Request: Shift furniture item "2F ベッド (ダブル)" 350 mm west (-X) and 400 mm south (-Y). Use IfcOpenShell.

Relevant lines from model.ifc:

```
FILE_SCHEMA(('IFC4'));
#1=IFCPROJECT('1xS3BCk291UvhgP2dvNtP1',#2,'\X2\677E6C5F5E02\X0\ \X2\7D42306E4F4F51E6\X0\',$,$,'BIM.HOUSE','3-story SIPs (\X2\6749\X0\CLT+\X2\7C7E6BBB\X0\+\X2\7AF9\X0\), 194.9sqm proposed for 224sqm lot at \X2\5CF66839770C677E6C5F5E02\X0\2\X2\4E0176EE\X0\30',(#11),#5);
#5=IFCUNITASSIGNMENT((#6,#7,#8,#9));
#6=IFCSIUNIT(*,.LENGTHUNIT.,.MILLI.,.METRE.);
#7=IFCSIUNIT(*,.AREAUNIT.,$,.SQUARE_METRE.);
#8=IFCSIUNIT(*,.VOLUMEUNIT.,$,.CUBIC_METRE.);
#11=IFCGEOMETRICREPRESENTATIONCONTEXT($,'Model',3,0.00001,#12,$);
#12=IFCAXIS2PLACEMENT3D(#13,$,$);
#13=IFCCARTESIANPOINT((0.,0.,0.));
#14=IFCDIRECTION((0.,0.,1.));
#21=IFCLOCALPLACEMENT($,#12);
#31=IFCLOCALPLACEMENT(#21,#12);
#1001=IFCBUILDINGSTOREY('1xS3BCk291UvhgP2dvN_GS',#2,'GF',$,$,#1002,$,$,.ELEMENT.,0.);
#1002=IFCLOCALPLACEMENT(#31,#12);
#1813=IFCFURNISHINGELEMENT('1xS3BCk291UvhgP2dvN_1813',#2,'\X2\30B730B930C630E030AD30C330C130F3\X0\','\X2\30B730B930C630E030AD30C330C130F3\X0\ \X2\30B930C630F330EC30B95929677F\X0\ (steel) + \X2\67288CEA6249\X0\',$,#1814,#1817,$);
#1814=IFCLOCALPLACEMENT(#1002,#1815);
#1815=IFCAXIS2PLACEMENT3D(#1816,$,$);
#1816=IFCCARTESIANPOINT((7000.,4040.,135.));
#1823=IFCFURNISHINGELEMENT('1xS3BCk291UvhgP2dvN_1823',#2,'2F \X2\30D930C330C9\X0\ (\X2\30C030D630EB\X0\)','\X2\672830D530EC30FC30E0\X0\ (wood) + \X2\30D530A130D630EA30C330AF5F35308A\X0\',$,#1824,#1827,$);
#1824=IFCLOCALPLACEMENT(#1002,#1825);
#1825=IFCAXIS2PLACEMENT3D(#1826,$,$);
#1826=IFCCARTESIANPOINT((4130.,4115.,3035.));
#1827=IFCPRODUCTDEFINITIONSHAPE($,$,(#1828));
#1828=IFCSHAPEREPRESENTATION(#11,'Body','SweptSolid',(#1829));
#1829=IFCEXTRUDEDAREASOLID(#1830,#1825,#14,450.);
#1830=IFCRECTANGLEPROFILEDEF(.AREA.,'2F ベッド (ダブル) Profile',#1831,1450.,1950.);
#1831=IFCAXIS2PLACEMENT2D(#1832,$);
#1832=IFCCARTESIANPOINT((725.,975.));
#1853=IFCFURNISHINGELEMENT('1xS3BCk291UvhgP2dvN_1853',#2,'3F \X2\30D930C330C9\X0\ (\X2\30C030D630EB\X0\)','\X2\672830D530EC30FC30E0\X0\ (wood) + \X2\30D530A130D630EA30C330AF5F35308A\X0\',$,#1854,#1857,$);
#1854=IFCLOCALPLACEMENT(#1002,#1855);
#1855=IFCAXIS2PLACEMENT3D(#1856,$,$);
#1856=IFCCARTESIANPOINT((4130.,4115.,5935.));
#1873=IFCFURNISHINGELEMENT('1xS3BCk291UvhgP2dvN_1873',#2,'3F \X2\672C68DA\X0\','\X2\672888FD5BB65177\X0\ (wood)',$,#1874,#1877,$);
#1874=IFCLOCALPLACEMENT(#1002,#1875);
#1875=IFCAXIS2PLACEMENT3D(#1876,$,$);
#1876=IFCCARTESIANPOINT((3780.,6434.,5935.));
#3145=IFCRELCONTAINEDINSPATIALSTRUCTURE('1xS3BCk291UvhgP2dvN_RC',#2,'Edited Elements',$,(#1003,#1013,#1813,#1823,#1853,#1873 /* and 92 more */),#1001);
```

```python
import ifcopenshell
import ifcopenshell.api.geometry
import ifcopenshell.util.placement

model = ifcopenshell.open("model.ifc")

item = model.by_id(1823)
matrix = ifcopenshell.util.placement.get_local_placement(item.ObjectPlacement)
matrix[0, 3] -= 350.0
matrix[1, 3] -= 400.0
ifcopenshell.api.geometry.edit_object_placement(model, product=item, matrix=matrix, is_si=False)

print(ifcopenshell.util.placement.get_local_placement(item.ObjectPlacement).round(3) + 0.0)

model.write("model_edited.ifc")
```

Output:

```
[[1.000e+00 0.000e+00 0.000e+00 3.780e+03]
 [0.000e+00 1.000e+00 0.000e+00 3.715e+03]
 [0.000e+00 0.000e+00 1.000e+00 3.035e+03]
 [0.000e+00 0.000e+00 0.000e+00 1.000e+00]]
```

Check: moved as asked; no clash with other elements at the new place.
